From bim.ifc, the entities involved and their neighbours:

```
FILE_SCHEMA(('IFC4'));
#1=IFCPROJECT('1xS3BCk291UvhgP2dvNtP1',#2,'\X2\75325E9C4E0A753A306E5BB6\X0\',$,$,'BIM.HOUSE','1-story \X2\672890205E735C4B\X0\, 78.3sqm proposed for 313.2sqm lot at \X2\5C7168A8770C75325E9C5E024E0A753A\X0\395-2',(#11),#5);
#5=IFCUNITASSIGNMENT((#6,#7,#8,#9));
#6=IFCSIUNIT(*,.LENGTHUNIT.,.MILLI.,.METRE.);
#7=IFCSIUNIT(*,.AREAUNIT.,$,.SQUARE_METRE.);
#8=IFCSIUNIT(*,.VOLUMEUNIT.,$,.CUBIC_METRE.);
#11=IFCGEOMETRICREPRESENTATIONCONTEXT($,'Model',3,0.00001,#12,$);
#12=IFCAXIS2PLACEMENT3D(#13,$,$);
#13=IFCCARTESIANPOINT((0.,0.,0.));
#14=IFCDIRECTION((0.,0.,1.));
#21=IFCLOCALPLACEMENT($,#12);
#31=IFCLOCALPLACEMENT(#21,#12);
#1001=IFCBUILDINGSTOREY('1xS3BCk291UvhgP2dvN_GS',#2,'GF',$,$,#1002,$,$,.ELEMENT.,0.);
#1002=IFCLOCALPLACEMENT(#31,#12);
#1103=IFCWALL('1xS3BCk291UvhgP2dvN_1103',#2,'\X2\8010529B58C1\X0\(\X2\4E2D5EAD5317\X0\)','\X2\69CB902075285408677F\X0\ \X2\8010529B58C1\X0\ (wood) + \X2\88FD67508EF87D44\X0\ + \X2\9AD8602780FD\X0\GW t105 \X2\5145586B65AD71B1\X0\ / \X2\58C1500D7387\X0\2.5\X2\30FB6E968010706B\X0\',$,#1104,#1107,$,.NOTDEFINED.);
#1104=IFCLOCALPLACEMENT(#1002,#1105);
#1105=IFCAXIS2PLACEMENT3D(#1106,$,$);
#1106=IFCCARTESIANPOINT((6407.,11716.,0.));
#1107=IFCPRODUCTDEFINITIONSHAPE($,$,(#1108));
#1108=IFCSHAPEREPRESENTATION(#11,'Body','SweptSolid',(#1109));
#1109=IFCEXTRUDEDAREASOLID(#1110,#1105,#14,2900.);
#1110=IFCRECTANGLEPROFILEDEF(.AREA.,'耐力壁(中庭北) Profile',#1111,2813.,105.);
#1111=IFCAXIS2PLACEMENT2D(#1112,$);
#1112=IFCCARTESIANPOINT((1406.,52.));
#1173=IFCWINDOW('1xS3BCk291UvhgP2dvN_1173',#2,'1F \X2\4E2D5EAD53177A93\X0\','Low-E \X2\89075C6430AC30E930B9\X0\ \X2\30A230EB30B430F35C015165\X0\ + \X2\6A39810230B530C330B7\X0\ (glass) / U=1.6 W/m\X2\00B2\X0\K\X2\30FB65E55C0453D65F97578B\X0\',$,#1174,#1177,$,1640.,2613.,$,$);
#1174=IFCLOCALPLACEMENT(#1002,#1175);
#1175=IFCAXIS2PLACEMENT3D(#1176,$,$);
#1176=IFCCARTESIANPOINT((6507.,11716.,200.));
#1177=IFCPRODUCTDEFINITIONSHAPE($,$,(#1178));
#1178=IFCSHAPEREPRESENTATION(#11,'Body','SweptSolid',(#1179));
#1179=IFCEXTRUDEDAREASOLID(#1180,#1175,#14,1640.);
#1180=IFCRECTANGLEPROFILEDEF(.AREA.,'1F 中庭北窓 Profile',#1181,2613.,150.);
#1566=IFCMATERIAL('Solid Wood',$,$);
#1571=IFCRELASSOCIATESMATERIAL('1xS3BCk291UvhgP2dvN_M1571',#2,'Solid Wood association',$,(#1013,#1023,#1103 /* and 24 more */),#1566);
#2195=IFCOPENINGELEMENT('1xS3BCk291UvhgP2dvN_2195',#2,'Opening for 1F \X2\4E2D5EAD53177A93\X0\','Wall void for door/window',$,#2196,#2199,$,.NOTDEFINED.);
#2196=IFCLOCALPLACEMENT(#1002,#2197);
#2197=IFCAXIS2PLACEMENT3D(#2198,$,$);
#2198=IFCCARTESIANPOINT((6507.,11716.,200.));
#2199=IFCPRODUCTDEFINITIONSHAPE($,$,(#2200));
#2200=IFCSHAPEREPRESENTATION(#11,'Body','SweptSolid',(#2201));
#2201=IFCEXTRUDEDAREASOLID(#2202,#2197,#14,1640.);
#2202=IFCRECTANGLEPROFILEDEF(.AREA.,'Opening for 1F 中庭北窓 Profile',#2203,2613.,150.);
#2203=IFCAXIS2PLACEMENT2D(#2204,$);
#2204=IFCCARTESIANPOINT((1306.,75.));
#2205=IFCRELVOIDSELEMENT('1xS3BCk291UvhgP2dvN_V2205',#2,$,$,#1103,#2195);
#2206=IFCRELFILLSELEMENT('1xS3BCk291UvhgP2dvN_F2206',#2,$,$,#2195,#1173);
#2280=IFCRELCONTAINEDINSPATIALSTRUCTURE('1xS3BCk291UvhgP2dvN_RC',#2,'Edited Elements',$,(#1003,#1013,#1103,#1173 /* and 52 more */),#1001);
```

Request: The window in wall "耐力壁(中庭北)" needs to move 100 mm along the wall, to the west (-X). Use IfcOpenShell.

```python
import ifcopenshell
import ifcopenshell.api.geometry
import ifcopenshell.util.placement

model = ifcopenshell.open("bim.ifc")

window = model.by_id(1173)
opening = window.FillsVoids[0].RelatingOpeningElement
wall = opening.VoidsElements[0].RelatingBuildingElement

wall_matrix = ifcopenshell.util.placement.get_local_placement(wall.ObjectPlacement)
shift = wall_matrix[:3, 0] * -100.0
before = ifcopenshell.util.placement.get_local_placement(window.ObjectPlacement)[:3, 3].copy()

# The window is not placed relative to its opening, so move both.
for product in (opening, window):
    matrix = ifcopenshell.util.placement.get_local_placement(product.ObjectPlacement)
    matrix[:3, 3] += shift
    ifcopenshell.api.geometry.edit_object_placement(model, product=product, matrix=matrix, is_si=False)

after = ifcopenshell.util.placement.get_local_placement(window.ObjectPlacement)[:3, 3]
print("window moved by", (after - before).round(3) + 0.0)

model.write("bim_v2.ifc")
```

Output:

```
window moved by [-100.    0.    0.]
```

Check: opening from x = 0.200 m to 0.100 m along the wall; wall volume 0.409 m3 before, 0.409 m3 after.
